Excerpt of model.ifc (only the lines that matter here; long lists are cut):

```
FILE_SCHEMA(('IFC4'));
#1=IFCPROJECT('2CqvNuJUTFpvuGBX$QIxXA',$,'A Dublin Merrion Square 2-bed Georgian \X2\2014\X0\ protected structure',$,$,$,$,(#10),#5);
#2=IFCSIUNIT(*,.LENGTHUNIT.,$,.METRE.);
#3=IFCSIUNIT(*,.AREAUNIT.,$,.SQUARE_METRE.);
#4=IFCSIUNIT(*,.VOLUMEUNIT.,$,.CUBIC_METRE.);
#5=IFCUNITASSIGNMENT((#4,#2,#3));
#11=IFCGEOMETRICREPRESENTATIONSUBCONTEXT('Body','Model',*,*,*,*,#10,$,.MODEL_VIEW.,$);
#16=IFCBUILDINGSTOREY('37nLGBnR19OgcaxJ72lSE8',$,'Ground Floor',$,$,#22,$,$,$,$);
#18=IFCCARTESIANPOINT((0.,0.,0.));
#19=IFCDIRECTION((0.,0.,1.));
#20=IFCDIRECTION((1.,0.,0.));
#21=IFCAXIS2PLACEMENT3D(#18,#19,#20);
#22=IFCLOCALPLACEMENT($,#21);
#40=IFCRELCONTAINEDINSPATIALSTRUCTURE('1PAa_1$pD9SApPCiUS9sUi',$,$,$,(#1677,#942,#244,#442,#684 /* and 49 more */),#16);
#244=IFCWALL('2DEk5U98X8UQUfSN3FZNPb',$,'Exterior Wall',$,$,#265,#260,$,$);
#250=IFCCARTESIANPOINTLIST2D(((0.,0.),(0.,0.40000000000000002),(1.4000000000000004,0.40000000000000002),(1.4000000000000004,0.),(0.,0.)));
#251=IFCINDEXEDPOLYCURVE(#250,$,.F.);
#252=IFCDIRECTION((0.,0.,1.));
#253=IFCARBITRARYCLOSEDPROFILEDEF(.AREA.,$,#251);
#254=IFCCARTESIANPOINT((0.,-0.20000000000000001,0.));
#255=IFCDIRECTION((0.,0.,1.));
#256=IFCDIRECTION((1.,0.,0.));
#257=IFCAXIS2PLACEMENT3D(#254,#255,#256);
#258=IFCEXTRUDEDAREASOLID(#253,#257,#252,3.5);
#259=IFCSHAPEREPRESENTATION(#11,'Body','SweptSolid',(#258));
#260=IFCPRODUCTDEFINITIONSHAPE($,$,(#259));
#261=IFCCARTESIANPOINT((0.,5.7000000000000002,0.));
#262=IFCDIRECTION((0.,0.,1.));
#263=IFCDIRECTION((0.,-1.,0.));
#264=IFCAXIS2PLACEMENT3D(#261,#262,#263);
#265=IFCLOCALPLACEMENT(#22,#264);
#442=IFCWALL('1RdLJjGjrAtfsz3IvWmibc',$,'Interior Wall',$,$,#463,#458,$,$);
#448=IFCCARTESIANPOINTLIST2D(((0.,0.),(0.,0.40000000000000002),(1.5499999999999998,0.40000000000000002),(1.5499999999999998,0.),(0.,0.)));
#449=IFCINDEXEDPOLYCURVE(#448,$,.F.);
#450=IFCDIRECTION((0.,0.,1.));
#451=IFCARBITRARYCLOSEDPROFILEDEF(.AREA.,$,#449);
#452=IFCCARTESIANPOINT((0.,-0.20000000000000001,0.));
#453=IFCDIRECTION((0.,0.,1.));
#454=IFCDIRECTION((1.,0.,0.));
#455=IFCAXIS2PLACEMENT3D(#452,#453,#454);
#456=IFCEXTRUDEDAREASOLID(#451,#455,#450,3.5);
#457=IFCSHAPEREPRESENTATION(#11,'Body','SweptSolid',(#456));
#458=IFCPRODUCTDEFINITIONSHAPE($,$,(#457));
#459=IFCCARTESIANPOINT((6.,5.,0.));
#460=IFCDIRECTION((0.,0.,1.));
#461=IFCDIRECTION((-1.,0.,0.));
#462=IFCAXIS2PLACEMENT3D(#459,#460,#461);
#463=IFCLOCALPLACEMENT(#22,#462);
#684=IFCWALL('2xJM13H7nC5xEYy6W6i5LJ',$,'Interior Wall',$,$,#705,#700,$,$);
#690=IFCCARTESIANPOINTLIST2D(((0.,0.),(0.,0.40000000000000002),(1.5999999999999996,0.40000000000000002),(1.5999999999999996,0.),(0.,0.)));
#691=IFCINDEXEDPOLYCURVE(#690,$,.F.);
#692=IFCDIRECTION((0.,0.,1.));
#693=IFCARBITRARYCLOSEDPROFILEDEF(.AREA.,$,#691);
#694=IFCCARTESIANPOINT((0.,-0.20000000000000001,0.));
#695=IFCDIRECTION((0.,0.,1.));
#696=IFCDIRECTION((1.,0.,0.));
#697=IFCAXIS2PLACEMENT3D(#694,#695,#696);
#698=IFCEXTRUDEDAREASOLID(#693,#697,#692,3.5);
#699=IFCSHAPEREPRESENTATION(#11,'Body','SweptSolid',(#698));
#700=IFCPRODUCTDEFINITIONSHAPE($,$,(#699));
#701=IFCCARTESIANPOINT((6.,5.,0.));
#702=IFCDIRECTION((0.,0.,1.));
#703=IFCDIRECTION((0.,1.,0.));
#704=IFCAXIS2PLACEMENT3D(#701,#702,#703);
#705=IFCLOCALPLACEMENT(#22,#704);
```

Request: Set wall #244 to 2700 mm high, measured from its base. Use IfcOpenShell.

```python
import ifcopenshell
import ifcopenshell.geom
import ifcopenshell.util.representation
import ifcopenshell.util.shape

model = ifcopenshell.open("model.ifc")
settings = ifcopenshell.geom.settings()


def volume(element):
    """Net volume in cubic metres, openings subtracted."""
    shape = ifcopenshell.geom.create_shape(settings, element)
    return ifcopenshell.util.shape.get_volume(shape.geometry)


wall = model.by_guid("2DEk5U98X8UQUfSN3FZNPb")
before = volume(wall)

body = ifcopenshell.util.representation.get_representation(wall, "Model", "Body")
solid = body.Items[0]
old_height = solid.Depth
solid.Depth = 2.7
after = volume(wall)

print(f"height {old_height:g} -> {solid.Depth:g}, volume {before:.3f} -> {after:.3f} m3")

model.write("model_rev.ifc")
```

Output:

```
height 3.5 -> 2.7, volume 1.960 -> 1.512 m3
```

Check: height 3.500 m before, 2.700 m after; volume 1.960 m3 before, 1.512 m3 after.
